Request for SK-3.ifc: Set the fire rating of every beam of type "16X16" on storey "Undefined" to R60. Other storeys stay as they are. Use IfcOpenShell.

First a look at what the model holds.

```python
import ifcopenshell
import ifcopenshell.util.element

model = ifcopenshell.open("SK-3.ifc")
print(model.schema)
storey = next(s for s in model.by_type("IfcBuildingStorey") if s.Name == "Undefined")
beams = [e for e in ifcopenshell.util.element.get_decomposition(storey) if e.is_a("IfcBeam")]
seen = {}
for e in beams:
    element_type = ifcopenshell.util.element.get_type(e)
    key = (element_type.Name if element_type != e and element_type else None, ifcopenshell.util.element.get_pset(e, "Pset_BeamCommon", "FireRating"))
    seen[key] = seen.get(key, 0) + 1
for (name, value), count in sorted(seen.items(), key=str):
    print(count, "x", name, "|", value)
```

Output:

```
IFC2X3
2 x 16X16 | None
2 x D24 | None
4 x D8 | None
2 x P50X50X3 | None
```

```python
import ifcopenshell
import ifcopenshell.api.pset
import ifcopenshell.util.element

model = ifcopenshell.open("SK-3.ifc")

storey = next(s for s in model.by_type("IfcBuildingStorey") if s.Name == "Undefined")
beams = [e for e in ifcopenshell.util.element.get_decomposition(storey) if e.is_a("IfcBeam")]

count = 0
for e in beams:
    element_type = ifcopenshell.util.element.get_type(e)
    if element_type in (None, e) or element_type.Name != "16X16":
        continue
    found = ifcopenshell.util.element.get_pset(e, "Pset_BeamCommon", should_inherit=False)
    if found:
        pset = model.by_id(found["id"])
        if len(ifcopenshell.util.element.get_elements_by_pset(pset)) > 1:
            pset = ifcopenshell.api.pset.unshare_pset(model, products=[e], pset=pset)[0]
    else:
        pset = ifcopenshell.api.pset.add_pset(model, product=e, name="Pset_BeamCommon")
    ifcopenshell.api.pset.edit_pset(model, pset=pset, properties={"FireRating": "R60"})
    count += 1

print(count, "beams updated")

model.write("SK-3_rev.ifc")
```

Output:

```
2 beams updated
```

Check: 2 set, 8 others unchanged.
